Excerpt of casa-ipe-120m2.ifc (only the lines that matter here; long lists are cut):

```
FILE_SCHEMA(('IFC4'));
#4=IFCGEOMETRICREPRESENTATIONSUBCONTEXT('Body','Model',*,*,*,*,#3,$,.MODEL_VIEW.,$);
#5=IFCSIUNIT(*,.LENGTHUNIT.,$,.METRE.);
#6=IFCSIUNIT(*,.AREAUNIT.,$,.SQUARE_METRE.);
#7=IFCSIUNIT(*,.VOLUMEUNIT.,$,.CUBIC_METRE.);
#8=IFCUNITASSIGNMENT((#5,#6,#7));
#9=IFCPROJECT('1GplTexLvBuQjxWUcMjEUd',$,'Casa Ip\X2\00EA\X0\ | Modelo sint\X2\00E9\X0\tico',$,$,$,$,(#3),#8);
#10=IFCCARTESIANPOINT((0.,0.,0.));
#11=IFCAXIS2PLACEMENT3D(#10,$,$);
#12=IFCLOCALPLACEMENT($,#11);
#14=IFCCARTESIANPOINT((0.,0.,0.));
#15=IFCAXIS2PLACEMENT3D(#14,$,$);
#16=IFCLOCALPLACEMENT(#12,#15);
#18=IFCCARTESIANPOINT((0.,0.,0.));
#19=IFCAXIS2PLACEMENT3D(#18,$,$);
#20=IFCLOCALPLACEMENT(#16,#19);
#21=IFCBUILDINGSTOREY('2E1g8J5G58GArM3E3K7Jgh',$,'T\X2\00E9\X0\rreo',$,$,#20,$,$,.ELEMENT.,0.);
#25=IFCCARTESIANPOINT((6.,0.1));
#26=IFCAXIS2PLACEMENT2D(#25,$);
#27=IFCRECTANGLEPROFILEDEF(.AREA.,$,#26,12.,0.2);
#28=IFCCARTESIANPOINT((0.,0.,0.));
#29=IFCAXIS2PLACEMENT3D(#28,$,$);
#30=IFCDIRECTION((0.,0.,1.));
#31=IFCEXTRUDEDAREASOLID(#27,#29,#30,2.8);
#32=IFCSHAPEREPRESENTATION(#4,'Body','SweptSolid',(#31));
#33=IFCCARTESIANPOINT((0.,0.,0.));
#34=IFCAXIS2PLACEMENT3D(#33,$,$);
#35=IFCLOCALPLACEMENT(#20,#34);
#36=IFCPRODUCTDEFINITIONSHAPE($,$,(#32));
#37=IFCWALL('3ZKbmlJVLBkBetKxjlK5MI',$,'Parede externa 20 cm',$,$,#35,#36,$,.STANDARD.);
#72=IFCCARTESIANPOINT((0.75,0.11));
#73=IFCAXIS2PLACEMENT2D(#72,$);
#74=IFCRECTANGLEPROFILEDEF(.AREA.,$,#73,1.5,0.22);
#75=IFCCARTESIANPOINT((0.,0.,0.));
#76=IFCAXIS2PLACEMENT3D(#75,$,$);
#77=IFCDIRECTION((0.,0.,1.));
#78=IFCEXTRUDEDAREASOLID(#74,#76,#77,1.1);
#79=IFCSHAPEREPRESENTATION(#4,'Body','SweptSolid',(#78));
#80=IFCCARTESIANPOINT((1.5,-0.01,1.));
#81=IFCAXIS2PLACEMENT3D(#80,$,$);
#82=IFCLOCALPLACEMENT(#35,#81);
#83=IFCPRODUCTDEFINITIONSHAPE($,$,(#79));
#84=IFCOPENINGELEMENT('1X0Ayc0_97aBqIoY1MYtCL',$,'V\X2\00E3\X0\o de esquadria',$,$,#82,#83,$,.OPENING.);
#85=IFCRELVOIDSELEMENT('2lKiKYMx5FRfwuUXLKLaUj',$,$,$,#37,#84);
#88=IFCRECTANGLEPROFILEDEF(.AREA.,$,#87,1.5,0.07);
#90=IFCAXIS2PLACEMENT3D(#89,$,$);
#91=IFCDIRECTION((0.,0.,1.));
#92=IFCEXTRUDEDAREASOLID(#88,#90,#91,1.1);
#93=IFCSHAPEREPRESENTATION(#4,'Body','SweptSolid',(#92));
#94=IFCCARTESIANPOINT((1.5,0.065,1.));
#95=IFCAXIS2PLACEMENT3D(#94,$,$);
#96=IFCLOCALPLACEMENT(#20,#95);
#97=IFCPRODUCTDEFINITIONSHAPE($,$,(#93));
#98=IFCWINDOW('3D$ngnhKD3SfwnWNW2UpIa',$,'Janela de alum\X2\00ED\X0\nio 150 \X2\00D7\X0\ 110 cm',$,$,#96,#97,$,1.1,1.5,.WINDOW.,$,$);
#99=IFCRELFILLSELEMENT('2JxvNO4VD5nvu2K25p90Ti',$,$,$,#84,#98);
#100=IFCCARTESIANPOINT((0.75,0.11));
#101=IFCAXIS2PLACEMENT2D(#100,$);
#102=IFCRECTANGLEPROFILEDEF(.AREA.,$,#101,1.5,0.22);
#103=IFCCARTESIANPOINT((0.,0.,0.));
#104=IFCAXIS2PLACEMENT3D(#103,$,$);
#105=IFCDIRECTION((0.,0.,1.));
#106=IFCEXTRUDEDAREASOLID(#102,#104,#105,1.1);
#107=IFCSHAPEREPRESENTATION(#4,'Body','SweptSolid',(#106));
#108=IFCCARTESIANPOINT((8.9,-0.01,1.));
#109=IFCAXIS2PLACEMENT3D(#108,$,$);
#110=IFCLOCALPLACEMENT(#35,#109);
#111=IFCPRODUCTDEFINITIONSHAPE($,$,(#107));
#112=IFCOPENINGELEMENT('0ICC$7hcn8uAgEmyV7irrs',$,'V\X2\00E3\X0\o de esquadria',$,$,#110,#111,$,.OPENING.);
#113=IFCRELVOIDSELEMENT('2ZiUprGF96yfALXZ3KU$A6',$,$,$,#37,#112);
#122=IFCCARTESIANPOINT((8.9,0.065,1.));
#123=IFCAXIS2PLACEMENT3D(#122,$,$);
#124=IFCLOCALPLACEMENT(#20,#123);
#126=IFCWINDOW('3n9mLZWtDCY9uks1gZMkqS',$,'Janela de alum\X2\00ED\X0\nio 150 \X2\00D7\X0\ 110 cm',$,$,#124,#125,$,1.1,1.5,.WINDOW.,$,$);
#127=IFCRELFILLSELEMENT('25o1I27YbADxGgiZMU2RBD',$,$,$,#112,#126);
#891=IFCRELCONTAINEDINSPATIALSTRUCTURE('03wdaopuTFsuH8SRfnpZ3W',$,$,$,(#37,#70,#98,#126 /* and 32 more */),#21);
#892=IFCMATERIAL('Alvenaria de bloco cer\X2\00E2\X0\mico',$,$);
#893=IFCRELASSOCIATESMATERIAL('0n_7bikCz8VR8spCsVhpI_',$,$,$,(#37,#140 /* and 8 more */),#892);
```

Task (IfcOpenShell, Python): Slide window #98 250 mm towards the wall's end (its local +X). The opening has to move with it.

```python
import ifcopenshell
import ifcopenshell.api.geometry
import ifcopenshell.util.placement

model = ifcopenshell.open("casa-ipe-120m2.ifc")

window = model.by_guid("3D$ngnhKD3SfwnWNW2UpIa")
opening = window.FillsVoids[0].RelatingOpeningElement
wall = opening.VoidsElements[0].RelatingBuildingElement

wall_matrix = ifcopenshell.util.placement.get_local_placement(wall.ObjectPlacement)
shift = wall_matrix[:3, 0] * 0.25
before = ifcopenshell.util.placement.get_local_placement(window.ObjectPlacement)[:3, 3].copy()

# The window is not placed relative to its opening, so move both.
for product in (opening, window):
    matrix = ifcopenshell.util.placement.get_local_placement(product.ObjectPlacement)
    matrix[:3, 3] += shift
    ifcopenshell.api.geometry.edit_object_placement(model, product=product, matrix=matrix, is_si=False)

after = ifcopenshell.util.placement.get_local_placement(window.ObjectPlacement)[:3, 3]
print("window moved by", (after - before).round(3) + 0.0)

model.write("casa-ipe-120m2_edited.ifc")
```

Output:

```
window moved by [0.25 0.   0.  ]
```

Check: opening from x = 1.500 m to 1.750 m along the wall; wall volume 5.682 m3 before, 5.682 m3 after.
